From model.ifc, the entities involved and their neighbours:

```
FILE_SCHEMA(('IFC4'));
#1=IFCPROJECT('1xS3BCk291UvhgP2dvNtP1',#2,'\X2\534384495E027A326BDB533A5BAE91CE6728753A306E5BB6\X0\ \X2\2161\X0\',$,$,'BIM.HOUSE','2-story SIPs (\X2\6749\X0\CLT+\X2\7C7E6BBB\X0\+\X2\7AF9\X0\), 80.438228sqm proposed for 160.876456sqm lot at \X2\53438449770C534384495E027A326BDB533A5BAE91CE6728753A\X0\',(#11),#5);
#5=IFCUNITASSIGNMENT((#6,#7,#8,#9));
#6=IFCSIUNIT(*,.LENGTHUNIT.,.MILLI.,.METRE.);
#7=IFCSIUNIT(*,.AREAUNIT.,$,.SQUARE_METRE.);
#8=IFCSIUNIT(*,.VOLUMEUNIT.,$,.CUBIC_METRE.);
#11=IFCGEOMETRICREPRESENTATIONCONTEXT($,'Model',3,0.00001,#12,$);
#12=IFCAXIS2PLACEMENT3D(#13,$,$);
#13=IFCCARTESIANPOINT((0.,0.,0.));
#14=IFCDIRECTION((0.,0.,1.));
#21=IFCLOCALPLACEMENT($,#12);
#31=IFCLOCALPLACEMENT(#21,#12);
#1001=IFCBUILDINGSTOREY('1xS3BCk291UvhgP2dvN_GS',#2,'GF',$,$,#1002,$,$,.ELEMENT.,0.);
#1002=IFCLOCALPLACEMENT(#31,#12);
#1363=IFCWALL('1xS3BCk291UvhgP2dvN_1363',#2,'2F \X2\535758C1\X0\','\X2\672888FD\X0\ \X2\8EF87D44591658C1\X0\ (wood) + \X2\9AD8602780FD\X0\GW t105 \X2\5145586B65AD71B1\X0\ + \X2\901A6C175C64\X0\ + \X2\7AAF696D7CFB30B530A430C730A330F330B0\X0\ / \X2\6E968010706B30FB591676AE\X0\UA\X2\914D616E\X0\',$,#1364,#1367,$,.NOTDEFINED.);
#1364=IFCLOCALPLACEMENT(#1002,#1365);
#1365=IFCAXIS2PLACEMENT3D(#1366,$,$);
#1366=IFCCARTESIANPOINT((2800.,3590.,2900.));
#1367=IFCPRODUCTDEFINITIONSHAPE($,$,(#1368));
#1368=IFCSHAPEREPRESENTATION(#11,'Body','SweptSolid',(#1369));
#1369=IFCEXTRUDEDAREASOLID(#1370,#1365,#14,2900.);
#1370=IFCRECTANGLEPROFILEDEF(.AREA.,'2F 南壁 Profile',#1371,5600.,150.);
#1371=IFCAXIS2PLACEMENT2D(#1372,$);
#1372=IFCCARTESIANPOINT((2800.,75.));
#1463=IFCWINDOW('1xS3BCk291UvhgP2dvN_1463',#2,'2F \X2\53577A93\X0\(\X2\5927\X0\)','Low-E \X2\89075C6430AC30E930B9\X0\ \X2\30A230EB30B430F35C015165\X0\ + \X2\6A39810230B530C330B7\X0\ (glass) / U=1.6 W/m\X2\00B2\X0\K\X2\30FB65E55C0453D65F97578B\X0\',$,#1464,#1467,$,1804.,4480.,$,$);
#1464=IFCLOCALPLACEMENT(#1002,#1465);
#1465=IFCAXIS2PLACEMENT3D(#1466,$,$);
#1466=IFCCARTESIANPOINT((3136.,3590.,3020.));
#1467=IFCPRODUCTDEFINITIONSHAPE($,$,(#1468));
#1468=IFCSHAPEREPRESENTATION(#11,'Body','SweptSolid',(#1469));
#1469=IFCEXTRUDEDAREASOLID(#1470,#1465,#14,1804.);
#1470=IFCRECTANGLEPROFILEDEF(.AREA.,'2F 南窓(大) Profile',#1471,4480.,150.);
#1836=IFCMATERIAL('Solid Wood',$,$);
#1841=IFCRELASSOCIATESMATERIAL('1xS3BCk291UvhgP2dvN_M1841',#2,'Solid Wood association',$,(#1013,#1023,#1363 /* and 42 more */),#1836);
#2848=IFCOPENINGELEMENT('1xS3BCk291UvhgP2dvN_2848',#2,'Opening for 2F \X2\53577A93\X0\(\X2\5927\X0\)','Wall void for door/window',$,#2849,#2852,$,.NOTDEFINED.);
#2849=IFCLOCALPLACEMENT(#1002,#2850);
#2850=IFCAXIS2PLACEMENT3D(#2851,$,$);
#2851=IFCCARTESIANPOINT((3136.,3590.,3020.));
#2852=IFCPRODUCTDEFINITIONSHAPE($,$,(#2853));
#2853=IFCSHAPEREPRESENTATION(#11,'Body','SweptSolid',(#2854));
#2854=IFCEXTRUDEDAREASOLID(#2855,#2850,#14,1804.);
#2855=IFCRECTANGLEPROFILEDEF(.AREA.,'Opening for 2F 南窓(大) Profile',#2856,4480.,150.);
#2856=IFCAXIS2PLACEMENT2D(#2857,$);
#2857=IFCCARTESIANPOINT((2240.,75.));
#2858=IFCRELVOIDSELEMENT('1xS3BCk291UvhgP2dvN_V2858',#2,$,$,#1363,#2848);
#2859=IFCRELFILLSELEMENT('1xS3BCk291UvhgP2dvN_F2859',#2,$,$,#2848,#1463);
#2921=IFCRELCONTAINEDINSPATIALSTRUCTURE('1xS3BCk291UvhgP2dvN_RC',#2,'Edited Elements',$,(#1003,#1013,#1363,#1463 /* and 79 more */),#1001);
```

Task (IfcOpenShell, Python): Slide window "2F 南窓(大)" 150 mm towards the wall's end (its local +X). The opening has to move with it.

```python
import ifcopenshell
import ifcopenshell.api.geometry
import ifcopenshell.util.placement
import ifcopenshell.util.unit

model = ifcopenshell.open("model.ifc")
unit_scale = ifcopenshell.util.unit.calculate_unit_scale(model)

window = model.by_guid("1xS3BCk291UvhgP2dvN_1463")
opening = window.FillsVoids[0].RelatingOpeningElement
wall = opening.VoidsElements[0].RelatingBuildingElement

wall_matrix = ifcopenshell.util.placement.get_local_placement(wall.ObjectPlacement)
shift = wall_matrix[:3, 0] * 0.15 / unit_scale
before = ifcopenshell.util.placement.get_local_placement(window.ObjectPlacement)[:3, 3].copy()

# The window is not placed relative to its opening, so move both.
for product in (opening, window):
    matrix = ifcopenshell.util.placement.get_local_placement(product.ObjectPlacement)
    matrix[:3, 3] += shift
    ifcopenshell.api.geometry.edit_object_placement(model, product=product, matrix=matrix, is_si=False)

after = ifcopenshell.util.placement.get_local_placement(window.ObjectPlacement)[:3, 3]
print("window moved by", (after - before).round(3) + 0.0)

model.write("model-out.ifc")
```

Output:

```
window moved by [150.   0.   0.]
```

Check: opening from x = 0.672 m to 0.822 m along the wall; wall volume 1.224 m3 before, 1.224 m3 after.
